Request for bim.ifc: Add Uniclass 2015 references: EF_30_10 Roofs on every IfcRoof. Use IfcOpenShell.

First a look at what the model holds.

```python
import ifcopenshell

model = ifcopenshell.open("bim.ifc")
print(model.schema)
print("classifications:", [c.Name for c in model.by_type("IfcClassification")])
for ifc_class in ("IfcDoor", "IfcRoof", "IfcStair", "IfcWall", "IfcWindow"):
    print(ifc_class, len(model.by_type(ifc_class)))
```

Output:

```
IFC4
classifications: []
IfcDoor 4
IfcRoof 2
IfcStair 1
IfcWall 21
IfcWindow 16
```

```python
import ifcopenshell
import ifcopenshell.api.classification

model = ifcopenshell.open("bim.ifc")

system = ifcopenshell.api.classification.add_classification(model, classification="Uniclass 2015")

codes = {
    "IfcRoof": ("EF_30_10", "Roofs"),
}
for ifc_class, (code, name) in codes.items():
    products = model.by_type(ifc_class)
    ifcopenshell.api.classification.add_reference(
        model, products=products, classification=system, identification=code, name=name
    )
    print(code, len(products))

model.write("bim-out.ifc")
```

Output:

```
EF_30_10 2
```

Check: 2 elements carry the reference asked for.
